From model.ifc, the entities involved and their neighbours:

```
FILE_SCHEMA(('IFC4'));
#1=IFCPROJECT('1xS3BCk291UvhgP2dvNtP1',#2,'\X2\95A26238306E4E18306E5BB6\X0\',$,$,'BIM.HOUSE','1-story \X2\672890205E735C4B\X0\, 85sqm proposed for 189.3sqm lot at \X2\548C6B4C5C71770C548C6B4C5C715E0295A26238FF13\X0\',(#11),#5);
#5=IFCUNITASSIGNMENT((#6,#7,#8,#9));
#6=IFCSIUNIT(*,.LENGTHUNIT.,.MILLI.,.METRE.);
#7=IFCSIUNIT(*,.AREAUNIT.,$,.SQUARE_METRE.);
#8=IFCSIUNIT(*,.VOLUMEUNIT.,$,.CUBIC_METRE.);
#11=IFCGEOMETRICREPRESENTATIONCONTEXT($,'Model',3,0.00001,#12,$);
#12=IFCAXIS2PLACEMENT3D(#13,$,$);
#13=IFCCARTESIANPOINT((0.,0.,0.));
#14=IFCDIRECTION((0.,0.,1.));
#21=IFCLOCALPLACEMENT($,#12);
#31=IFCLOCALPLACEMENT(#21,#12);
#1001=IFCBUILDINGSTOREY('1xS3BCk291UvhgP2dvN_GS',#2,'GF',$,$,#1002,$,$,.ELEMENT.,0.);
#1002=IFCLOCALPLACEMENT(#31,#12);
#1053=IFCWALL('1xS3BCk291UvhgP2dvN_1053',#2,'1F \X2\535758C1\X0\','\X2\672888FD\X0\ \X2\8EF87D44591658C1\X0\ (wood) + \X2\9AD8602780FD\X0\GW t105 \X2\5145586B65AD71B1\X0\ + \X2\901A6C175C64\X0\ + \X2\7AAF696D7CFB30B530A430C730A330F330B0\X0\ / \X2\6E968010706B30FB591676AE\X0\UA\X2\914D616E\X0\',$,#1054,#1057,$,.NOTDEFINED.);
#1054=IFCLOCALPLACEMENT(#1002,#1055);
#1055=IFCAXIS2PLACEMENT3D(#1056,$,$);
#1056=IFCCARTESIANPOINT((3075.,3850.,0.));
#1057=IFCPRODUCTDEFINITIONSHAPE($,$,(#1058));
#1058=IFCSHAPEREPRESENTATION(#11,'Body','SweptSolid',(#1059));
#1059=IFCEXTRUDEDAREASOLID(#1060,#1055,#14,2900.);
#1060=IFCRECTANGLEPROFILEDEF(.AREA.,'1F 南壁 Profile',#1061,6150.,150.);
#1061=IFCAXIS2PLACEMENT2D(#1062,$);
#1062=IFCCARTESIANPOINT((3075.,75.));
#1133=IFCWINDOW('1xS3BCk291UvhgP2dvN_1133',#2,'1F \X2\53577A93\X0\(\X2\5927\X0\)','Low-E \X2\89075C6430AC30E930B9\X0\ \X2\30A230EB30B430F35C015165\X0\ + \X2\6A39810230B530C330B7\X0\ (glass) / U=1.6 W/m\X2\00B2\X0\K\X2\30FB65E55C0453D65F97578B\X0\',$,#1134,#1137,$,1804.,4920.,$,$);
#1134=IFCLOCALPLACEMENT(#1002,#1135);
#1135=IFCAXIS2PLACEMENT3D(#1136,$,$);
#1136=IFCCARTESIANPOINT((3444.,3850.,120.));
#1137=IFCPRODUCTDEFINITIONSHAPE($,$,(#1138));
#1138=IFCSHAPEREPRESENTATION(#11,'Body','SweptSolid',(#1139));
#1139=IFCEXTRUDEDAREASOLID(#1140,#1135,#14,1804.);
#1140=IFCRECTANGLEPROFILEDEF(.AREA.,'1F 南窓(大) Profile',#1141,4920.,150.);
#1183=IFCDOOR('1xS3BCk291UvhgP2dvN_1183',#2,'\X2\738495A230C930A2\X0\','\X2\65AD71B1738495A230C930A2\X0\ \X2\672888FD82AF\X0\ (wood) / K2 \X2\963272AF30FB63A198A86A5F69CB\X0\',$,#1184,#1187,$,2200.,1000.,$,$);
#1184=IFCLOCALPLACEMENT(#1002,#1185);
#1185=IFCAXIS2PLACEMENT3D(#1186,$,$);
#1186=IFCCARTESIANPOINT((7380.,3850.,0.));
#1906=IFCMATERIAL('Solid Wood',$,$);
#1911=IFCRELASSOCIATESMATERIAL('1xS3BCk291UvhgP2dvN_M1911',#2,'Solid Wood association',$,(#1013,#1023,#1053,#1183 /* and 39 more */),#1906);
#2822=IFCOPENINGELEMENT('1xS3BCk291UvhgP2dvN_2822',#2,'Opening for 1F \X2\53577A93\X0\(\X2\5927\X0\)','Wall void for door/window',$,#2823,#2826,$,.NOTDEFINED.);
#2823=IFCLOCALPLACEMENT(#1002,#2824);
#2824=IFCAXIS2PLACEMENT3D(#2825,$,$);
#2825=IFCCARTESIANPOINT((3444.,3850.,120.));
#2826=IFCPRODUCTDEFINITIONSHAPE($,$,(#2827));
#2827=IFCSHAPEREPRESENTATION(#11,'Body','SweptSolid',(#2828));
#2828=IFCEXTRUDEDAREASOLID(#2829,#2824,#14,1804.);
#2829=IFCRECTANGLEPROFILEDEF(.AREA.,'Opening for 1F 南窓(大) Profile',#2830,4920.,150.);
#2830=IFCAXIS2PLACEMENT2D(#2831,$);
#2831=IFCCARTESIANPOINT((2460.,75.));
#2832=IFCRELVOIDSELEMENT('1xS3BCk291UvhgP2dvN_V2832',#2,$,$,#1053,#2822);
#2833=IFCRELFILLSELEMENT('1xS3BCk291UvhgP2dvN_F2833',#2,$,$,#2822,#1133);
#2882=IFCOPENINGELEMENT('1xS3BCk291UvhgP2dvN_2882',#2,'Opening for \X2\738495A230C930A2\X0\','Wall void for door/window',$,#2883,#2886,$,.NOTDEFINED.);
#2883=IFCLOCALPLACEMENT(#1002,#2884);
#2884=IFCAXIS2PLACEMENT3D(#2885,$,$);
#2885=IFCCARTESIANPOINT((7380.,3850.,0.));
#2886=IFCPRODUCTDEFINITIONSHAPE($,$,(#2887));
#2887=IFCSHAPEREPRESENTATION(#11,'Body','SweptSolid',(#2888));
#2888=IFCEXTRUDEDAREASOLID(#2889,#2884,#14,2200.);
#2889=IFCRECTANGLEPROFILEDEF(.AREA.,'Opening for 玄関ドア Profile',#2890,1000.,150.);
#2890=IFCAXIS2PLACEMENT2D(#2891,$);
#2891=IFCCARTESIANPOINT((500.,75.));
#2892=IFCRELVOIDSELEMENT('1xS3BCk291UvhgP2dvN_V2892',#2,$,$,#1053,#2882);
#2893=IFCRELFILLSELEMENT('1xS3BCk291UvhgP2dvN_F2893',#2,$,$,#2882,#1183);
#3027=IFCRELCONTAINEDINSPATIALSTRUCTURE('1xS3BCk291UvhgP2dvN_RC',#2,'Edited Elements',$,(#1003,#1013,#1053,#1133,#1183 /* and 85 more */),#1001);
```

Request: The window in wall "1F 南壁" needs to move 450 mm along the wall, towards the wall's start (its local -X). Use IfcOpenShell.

```python
import ifcopenshell
import ifcopenshell.api.geometry
import ifcopenshell.util.placement
import ifcopenshell.util.unit

model = ifcopenshell.open("model.ifc")
unit_scale = ifcopenshell.util.unit.calculate_unit_scale(model)

window = model.by_guid("1xS3BCk291UvhgP2dvN_1133")
opening = window.FillsVoids[0].RelatingOpeningElement
wall = opening.VoidsElements[0].RelatingBuildingElement

wall_matrix = ifcopenshell.util.placement.get_local_placement(wall.ObjectPlacement)
shift = wall_matrix[:3, 0] * -0.45 / unit_scale
before = ifcopenshell.util.placement.get_local_placement(window.ObjectPlacement)[:3, 3].copy()

# The window is not placed relative to its opening, so move both.
for product in (opening, window):
    matrix = ifcopenshell.util.placement.get_local_placement(product.ObjectPlacement)
    matrix[:3, 3] += shift
    ifcopenshell.api.geometry.edit_object_placement(model, product=product, matrix=matrix, is_si=False)

after = ifcopenshell.util.placement.get_local_placement(window.ObjectPlacement)[:3, 3]
print("window moved by", (after - before).round(3) + 0.0)

model.write("model_edited.ifc")
```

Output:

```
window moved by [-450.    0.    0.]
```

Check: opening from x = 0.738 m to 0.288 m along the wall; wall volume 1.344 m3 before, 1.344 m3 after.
